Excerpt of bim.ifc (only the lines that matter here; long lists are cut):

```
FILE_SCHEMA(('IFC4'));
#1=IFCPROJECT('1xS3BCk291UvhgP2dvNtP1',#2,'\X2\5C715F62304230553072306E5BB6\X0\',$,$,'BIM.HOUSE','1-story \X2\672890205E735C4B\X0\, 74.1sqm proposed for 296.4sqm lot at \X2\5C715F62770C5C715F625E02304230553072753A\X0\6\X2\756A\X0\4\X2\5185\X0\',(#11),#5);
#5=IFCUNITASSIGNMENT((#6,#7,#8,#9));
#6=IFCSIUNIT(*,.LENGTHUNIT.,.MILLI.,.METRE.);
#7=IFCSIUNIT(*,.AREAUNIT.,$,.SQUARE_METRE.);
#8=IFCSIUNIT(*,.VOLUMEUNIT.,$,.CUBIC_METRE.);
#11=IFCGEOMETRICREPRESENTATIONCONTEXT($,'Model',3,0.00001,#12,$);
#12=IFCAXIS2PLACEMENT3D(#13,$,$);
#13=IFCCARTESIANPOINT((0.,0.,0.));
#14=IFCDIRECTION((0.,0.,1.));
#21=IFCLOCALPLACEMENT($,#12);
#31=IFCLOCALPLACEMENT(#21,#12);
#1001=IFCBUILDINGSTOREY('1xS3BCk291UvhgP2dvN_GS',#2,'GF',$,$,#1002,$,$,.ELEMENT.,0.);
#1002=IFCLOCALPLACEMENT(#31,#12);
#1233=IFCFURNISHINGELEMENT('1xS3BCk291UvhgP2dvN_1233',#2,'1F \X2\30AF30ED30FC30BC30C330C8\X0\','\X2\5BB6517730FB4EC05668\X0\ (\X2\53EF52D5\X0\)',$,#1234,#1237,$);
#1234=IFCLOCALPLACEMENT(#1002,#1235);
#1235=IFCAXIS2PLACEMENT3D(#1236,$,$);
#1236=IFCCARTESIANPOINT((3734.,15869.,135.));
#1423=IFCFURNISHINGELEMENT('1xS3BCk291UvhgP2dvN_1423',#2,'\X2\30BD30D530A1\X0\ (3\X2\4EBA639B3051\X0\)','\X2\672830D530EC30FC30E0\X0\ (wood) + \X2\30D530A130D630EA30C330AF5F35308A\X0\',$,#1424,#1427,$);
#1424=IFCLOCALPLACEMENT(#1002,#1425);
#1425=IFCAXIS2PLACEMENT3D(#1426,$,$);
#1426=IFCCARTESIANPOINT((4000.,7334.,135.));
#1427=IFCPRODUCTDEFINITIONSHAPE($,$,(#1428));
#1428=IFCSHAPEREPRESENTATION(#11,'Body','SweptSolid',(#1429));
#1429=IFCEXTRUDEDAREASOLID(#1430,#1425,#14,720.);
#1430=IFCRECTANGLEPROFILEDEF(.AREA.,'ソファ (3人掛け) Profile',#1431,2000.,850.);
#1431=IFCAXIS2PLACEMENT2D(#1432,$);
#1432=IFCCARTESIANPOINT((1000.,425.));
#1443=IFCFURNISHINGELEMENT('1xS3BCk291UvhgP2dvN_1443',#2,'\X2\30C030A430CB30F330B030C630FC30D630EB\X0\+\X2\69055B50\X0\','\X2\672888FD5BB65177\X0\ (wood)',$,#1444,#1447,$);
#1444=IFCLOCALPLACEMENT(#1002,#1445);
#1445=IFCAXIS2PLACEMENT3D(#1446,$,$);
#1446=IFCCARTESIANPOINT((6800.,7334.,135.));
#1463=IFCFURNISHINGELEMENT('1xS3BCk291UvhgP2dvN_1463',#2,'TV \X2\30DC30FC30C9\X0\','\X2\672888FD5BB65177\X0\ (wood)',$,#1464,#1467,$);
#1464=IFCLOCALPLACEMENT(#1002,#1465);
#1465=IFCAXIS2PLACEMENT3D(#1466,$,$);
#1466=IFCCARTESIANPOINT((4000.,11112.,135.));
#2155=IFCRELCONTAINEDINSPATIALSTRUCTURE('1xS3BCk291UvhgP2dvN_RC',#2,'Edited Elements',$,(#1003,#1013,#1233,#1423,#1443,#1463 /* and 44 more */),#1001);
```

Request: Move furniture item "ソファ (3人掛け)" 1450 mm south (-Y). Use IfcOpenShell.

```python
import ifcopenshell
import ifcopenshell.api.geometry
import ifcopenshell.util.placement

model = ifcopenshell.open("bim.ifc")

item = model.by_guid("1xS3BCk291UvhgP2dvN_1423")
matrix = ifcopenshell.util.placement.get_local_placement(item.ObjectPlacement)
matrix[1, 3] -= 1450.0
ifcopenshell.api.geometry.edit_object_placement(model, product=item, matrix=matrix, is_si=False)

print(ifcopenshell.util.placement.get_local_placement(item.ObjectPlacement).round(3) + 0.0)

model.write("bim_updated.ifc")
```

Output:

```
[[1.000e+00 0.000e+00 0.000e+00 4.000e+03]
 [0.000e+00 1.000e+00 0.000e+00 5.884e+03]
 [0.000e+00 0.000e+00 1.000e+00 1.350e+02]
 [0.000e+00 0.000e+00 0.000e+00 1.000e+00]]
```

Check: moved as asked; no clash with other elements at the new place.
